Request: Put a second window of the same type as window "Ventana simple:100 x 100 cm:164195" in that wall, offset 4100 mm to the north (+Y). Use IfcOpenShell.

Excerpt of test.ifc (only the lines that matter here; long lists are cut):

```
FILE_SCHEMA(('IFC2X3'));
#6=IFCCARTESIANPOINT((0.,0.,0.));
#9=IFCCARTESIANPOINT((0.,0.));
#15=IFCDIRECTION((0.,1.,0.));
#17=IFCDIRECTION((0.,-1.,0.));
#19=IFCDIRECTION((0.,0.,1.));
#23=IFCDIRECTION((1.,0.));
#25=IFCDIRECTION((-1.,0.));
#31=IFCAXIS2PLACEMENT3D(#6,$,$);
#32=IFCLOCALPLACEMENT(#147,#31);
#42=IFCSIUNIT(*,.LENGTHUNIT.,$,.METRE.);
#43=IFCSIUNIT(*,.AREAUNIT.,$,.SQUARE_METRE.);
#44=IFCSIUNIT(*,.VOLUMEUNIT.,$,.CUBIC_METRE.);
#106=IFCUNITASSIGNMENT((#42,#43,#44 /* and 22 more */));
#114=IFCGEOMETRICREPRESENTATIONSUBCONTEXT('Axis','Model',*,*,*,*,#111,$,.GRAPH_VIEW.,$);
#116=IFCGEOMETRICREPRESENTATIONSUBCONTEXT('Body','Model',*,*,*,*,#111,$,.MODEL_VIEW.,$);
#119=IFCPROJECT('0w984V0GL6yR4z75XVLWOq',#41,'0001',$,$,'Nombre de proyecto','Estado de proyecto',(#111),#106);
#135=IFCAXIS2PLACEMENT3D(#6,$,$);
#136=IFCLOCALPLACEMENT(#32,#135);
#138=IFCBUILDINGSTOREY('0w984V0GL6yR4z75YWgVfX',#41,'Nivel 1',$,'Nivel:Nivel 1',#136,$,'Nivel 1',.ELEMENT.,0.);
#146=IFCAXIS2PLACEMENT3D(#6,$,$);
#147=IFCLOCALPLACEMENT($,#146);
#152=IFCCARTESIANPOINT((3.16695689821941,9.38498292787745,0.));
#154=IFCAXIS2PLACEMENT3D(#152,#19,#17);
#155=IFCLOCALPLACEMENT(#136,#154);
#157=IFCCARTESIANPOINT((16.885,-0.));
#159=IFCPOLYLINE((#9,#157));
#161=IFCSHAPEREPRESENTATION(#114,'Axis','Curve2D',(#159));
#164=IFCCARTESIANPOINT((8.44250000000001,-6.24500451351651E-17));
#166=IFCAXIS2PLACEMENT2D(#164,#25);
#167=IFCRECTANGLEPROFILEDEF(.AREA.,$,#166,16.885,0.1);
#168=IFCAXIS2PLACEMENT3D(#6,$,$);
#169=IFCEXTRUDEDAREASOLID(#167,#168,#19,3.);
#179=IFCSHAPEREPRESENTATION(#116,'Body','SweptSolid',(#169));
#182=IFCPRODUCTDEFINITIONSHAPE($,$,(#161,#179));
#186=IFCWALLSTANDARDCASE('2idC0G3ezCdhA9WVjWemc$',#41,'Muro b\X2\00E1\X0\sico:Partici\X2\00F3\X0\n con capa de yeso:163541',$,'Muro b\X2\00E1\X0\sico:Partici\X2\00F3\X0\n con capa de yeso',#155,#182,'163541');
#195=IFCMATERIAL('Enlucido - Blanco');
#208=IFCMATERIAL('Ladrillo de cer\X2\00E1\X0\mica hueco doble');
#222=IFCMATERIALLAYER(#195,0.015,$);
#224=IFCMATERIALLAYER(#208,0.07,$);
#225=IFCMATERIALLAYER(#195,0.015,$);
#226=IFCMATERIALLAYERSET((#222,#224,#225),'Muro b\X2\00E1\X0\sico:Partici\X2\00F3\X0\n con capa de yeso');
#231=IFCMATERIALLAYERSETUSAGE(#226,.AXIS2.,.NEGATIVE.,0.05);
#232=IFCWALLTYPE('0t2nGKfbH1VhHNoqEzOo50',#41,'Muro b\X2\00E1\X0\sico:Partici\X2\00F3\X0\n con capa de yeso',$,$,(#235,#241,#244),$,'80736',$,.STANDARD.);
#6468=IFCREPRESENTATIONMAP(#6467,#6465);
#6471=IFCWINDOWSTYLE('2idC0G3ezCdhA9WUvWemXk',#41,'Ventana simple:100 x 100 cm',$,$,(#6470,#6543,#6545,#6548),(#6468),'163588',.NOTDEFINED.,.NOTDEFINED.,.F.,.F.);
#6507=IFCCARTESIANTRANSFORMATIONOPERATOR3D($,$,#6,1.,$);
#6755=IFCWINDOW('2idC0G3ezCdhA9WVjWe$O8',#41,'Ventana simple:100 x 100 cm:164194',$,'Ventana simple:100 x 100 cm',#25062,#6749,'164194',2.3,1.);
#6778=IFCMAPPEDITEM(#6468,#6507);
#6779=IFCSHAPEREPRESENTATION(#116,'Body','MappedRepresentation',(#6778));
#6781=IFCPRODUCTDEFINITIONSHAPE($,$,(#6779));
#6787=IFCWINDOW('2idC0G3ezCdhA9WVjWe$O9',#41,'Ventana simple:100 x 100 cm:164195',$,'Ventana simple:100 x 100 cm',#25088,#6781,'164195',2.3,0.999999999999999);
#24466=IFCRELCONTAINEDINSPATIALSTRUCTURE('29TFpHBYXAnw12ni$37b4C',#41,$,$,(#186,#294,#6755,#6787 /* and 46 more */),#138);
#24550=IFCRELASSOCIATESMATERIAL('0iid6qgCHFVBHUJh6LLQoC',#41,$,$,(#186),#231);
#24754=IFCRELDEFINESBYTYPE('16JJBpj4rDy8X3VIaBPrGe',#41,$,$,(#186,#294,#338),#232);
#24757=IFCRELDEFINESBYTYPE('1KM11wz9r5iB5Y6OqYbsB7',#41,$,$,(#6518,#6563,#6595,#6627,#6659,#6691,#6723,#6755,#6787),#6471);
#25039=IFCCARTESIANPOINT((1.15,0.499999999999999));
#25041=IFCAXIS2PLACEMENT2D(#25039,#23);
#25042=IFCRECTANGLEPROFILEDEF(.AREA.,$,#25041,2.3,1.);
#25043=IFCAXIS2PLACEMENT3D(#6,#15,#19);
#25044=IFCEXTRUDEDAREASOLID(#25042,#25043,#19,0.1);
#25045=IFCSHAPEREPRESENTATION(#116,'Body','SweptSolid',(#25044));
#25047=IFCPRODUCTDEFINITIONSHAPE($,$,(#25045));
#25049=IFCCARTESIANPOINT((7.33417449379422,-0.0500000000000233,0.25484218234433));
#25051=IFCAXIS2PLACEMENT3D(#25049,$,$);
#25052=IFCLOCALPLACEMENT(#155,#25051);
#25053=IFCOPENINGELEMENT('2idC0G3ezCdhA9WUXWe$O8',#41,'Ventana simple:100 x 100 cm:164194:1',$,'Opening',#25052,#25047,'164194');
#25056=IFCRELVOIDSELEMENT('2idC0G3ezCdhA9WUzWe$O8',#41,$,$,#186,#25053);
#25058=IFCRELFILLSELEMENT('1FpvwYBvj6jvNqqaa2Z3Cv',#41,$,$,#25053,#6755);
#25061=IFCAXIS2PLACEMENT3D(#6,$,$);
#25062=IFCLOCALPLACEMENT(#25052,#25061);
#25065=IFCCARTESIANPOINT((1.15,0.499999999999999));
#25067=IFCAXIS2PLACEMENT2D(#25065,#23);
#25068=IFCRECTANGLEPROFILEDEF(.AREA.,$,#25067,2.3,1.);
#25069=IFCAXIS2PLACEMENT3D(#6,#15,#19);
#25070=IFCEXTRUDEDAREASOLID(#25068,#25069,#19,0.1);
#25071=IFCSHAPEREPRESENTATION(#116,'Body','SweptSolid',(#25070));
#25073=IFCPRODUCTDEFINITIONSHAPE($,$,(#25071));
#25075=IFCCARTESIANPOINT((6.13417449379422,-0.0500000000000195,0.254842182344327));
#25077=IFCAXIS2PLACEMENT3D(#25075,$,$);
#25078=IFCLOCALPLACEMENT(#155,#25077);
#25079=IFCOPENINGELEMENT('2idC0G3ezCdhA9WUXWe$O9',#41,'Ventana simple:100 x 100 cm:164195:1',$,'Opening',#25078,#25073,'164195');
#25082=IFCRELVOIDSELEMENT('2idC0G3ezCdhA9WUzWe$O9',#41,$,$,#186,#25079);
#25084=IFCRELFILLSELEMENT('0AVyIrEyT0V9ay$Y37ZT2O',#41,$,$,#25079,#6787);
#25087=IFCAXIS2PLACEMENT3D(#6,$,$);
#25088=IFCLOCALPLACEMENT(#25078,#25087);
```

```python
import ifcopenshell
import ifcopenshell.api.feature
import ifcopenshell.api.geometry
import ifcopenshell.api.root
import ifcopenshell.geom
import ifcopenshell.util.element
import ifcopenshell.util.placement
import ifcopenshell.util.shape
import ifcopenshell.util.unit

model = ifcopenshell.open("test.ifc")
unit_scale = ifcopenshell.util.unit.calculate_unit_scale(model)
settings = ifcopenshell.geom.settings()


def volume(element):
    """Net volume in cubic metres, openings subtracted."""
    shape = ifcopenshell.geom.create_shape(settings, element)
    return ifcopenshell.util.shape.get_volume(shape.geometry)


def reuse_history(source, copy):
    """copy_class also copies each property set's owner history, people and application; keep the originals."""
    for rel in copy.IsDefinedBy:
        if rel.is_a("IfcRelDefinesByProperties") and (history := rel.RelatingPropertyDefinition.OwnerHistory):
            rel.RelatingPropertyDefinition.OwnerHistory = source.OwnerHistory
            ifcopenshell.util.element.remove_deep2(model, history)


window = model.by_id(6787)
opening = window.FillsVoids[0].RelatingOpeningElement
wall = opening.VoidsElements[0].RelatingBuildingElement
before = volume(wall)
shift = ifcopenshell.util.placement.get_local_placement(wall.ObjectPlacement)[:3, 0] * -4.1 / unit_scale

# copy_class copies the void relationship, type, container and properties, but no geometry.
new_opening = ifcopenshell.api.root.copy_class(model, product=opening)
new_opening.Representation = ifcopenshell.util.element.copy_deep(
    model, opening.Representation, exclude=["IfcGeometricRepresentationContext", "IfcRepresentationMap"]
)
new_opening.Name = "Ventana simple:100 x 100 cm"
new_opening.Tag = None
new_window = ifcopenshell.api.root.copy_class(model, product=window)
new_window.Representation = ifcopenshell.util.element.copy_deep(
    model, window.Representation, exclude=["IfcGeometricRepresentationContext", "IfcRepresentationMap"]
)
new_window.Name = "Ventana simple:100 x 100 cm"
new_window.Tag = None
reuse_history(window, new_window)
fills = ifcopenshell.api.feature.add_filling(model, opening=new_opening, element=new_window)
fills.OwnerHistory = new_window.OwnerHistory  # required in IFC2X3

for old, new in ((opening, new_opening), (window, new_window)):
    matrix = ifcopenshell.util.placement.get_local_placement(old.ObjectPlacement)
    matrix[:3, 3] += shift
    ifcopenshell.api.geometry.edit_object_placement(model, product=new, matrix=matrix, is_si=False)

after = volume(wall)

print(f"wall volume {before:.3f} -> {after:.3f} m3")

model.write("test_v2.ifc")
```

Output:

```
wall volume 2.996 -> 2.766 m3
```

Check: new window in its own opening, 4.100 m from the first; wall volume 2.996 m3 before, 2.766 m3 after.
